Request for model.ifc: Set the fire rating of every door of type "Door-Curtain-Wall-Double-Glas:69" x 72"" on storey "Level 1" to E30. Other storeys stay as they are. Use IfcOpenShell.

First a look at what the model holds.

```python
import ifcopenshell
import ifcopenshell.util.element

model = ifcopenshell.open("model.ifc")
print(model.schema)
storey = next(s for s in model.by_type("IfcBuildingStorey") if s.Name == "Level 1")
doors = [e for e in ifcopenshell.util.element.get_decomposition(storey) if e.is_a("IfcDoor")]
seen = {}
for e in doors:
    element_type = ifcopenshell.util.element.get_type(e)
    key = (element_type.Name if element_type != e and element_type else None, ifcopenshell.util.element.get_pset(e, "Pset_DoorCommon", "FireRating"))
    seen[key] = seen.get(key, 0) + 1
for (name, value), count in sorted(seen.items(), key=str):
    print(count, "x", name, "|", value)
```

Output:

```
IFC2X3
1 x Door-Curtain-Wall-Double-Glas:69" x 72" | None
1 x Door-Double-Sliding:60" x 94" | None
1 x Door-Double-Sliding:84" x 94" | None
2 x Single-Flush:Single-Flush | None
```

```python
import ifcopenshell
import ifcopenshell.api.pset
import ifcopenshell.util.element

model = ifcopenshell.open("model.ifc")

storey = next(s for s in model.by_type("IfcBuildingStorey") if s.Name == "Level 1")
doors = [e for e in ifcopenshell.util.element.get_decomposition(storey) if e.is_a("IfcDoor")]

count = 0
for e in doors:
    element_type = ifcopenshell.util.element.get_type(e)
    if element_type in (None, e) or element_type.Name != 'Door-Curtain-Wall-Double-Glas:69" x 72"':
        continue
    # add_pset returns the element's existing set when there is one.
    pset = ifcopenshell.api.pset.add_pset(model, product=e, name="Pset_DoorCommon")
    ifcopenshell.api.pset.edit_pset(model, pset=pset, properties={"FireRating": "E30"})
    count += 1

print(count, "doors updated")

model.write("model_edited.ifc")
```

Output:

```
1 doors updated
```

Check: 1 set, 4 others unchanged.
